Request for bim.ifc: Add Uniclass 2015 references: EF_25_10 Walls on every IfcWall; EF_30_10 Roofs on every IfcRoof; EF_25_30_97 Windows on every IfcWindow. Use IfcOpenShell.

First a look at what the model holds.

```python
import ifcopenshell

model = ifcopenshell.open("bim.ifc")
print(model.schema)
print("classifications:", [c.Name for c in model.by_type("IfcClassification")])
for ifc_class in ("IfcDoor", "IfcRoof", "IfcStair", "IfcWall", "IfcWindow"):
    print(ifc_class, len(model.by_type(ifc_class)))
```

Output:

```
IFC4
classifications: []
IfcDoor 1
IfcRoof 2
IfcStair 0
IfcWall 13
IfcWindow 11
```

```python
import ifcopenshell
import ifcopenshell.api.classification

model = ifcopenshell.open("bim.ifc")

system = ifcopenshell.api.classification.add_classification(model, classification="Uniclass 2015")

codes = {
    "IfcWall": ("EF_25_10", "Walls"),
    "IfcRoof": ("EF_30_10", "Roofs"),
    "IfcWindow": ("EF_25_30_97", "Windows"),
}
for ifc_class, (code, name) in codes.items():
    products = model.by_type(ifc_class)
    ifcopenshell.api.classification.add_reference(
        model, products=products, classification=system, identification=code, name=name
    )
    print(code, len(products))

model.write("bim_edited.ifc")
```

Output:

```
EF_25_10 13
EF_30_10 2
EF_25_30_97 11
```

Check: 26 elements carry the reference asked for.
